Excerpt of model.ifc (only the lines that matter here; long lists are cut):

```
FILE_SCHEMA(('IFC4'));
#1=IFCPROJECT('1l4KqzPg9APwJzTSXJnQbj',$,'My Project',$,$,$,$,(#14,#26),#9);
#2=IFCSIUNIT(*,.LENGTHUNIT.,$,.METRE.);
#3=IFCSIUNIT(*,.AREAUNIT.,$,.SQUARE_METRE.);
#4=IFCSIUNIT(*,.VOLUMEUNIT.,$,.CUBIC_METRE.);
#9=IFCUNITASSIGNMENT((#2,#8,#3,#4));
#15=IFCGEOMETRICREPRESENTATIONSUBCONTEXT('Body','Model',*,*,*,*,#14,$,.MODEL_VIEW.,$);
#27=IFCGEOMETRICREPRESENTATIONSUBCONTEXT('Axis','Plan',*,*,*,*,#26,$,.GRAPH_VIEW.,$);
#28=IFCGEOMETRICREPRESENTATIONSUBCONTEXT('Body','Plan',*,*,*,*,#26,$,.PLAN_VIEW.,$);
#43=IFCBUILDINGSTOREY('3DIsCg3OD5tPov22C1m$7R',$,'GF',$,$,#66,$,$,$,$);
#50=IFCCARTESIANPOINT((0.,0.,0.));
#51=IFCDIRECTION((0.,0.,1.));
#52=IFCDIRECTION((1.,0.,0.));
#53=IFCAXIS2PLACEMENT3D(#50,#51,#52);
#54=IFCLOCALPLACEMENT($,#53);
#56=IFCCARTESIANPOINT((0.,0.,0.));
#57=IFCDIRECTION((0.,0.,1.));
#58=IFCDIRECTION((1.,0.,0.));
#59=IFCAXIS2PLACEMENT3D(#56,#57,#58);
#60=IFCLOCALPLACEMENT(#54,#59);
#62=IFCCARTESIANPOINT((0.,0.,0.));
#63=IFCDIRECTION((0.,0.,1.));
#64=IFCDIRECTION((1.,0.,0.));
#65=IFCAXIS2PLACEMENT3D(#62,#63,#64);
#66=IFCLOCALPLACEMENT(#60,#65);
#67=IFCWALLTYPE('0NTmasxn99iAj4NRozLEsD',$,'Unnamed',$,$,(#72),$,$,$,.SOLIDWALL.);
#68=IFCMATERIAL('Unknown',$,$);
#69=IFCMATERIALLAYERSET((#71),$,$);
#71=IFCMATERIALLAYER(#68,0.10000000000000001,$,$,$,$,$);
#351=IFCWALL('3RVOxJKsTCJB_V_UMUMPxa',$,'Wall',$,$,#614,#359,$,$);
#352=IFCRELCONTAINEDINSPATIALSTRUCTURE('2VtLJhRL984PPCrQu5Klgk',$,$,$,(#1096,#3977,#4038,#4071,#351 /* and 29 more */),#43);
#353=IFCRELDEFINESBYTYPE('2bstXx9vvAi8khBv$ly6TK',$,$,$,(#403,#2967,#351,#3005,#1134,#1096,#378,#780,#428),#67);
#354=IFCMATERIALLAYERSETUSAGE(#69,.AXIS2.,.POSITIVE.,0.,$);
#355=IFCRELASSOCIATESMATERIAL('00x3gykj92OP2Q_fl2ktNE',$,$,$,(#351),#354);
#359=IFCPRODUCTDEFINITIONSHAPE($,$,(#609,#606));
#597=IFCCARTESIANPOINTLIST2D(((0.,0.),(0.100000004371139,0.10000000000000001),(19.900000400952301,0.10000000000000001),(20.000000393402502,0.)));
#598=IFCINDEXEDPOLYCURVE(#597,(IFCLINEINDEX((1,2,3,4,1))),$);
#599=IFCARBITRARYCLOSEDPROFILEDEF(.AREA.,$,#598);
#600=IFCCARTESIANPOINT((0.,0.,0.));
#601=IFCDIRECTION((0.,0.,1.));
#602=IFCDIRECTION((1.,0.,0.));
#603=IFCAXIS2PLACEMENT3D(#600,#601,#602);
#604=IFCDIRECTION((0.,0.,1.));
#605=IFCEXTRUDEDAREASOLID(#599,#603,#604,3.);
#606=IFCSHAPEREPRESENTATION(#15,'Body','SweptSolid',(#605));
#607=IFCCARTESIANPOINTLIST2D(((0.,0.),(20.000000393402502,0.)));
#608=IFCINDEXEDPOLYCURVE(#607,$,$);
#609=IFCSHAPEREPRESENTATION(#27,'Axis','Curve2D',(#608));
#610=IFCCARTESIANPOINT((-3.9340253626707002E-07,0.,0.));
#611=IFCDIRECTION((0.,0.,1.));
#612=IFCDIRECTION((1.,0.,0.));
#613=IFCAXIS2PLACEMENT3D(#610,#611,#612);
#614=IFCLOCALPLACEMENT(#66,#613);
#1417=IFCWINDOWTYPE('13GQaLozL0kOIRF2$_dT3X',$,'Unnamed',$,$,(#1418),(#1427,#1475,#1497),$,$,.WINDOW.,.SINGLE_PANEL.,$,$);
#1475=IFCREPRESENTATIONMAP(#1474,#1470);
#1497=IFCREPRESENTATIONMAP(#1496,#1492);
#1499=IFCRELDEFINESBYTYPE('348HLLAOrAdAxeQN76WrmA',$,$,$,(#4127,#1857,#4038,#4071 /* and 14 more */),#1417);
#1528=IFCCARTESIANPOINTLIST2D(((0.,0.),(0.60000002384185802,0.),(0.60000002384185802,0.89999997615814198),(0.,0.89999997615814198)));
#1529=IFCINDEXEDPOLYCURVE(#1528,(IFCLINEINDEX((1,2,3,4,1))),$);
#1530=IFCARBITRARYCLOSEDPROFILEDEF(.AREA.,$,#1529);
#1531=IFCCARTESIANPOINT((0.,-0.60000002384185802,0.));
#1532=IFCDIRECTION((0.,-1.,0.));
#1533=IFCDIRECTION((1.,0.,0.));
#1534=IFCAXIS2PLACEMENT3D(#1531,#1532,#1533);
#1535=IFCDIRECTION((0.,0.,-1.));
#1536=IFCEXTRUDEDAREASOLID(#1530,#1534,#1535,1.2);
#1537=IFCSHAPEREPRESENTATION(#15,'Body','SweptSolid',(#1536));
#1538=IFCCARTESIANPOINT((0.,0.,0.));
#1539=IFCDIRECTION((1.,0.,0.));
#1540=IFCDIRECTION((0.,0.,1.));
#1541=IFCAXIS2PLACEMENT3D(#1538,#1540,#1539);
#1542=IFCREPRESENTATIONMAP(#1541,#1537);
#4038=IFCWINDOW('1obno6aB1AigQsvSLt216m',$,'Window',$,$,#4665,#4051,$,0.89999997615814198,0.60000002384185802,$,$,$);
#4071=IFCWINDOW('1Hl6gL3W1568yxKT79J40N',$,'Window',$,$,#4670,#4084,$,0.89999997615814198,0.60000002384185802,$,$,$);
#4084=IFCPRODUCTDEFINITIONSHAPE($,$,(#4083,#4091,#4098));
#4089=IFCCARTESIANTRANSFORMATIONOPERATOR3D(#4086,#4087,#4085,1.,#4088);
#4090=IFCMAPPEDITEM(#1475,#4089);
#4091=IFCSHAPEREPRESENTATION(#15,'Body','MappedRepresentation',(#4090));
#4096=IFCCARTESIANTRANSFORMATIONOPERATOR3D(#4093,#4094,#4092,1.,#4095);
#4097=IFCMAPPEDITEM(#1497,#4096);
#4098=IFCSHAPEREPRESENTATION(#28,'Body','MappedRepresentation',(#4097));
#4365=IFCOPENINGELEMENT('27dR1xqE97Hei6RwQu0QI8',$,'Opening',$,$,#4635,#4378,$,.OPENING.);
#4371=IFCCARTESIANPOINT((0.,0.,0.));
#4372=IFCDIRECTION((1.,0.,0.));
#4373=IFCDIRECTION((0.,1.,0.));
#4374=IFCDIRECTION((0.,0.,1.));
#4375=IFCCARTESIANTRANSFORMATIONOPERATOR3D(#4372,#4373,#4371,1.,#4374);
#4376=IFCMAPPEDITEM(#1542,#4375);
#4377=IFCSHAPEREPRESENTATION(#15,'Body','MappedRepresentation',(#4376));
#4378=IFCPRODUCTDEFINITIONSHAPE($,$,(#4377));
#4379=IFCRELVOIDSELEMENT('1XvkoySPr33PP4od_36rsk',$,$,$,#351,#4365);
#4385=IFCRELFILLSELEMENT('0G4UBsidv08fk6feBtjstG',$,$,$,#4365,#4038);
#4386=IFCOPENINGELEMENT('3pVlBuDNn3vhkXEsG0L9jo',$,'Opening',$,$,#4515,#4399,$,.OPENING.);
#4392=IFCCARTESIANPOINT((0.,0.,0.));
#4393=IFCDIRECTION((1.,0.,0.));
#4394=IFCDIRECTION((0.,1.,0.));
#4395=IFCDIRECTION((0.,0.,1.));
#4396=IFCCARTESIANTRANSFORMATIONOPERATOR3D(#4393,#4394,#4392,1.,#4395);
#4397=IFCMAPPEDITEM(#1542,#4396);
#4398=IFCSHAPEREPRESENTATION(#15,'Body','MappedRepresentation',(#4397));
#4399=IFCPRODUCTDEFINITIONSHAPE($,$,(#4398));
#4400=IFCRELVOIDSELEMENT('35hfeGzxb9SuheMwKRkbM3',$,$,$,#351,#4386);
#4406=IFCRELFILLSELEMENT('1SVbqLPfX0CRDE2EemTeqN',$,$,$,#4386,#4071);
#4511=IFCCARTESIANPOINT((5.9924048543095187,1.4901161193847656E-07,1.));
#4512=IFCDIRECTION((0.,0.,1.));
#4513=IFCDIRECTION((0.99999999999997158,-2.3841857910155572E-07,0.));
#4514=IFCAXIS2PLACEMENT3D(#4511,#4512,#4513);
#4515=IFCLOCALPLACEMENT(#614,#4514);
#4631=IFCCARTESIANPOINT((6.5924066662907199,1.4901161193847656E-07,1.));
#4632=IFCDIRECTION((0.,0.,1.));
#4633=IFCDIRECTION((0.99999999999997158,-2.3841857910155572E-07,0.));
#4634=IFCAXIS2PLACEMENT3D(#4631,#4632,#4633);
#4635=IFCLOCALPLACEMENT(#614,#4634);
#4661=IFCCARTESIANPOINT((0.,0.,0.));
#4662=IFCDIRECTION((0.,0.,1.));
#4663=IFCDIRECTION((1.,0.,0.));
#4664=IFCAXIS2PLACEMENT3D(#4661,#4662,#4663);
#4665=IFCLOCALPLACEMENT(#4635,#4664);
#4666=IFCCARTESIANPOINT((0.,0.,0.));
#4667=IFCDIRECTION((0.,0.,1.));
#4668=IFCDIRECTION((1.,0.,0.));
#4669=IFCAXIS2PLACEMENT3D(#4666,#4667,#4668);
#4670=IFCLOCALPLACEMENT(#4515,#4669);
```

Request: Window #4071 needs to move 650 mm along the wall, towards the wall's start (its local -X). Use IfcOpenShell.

```python
import ifcopenshell
import ifcopenshell.api.geometry
import ifcopenshell.util.placement
import ifcopenshell.util.unit

model = ifcopenshell.open("model.ifc")
unit_scale = ifcopenshell.util.unit.calculate_unit_scale(model)

window = model.by_guid("1Hl6gL3W1568yxKT79J40N")
opening = window.FillsVoids[0].RelatingOpeningElement
wall = opening.VoidsElements[0].RelatingBuildingElement

wall_matrix = ifcopenshell.util.placement.get_local_placement(wall.ObjectPlacement)
shift = wall_matrix[:3, 0] * -0.65 / unit_scale
before = ifcopenshell.util.placement.get_local_placement(window.ObjectPlacement)[:3, 3].copy()

# The window is placed relative to its opening, so it follows when the opening moves.
matrix = ifcopenshell.util.placement.get_local_placement(opening.ObjectPlacement)
matrix[:3, 3] += shift
ifcopenshell.api.geometry.edit_object_placement(
    model, product=opening, matrix=matrix, is_si=False, should_transform_children=True
)

after = ifcopenshell.util.placement.get_local_placement(window.ObjectPlacement)[:3, 3]
print("window moved by", (after - before).round(3) + 0.0)

model.write("model_edited.ifc")
```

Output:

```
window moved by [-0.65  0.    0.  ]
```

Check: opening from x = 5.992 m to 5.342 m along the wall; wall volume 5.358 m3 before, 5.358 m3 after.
